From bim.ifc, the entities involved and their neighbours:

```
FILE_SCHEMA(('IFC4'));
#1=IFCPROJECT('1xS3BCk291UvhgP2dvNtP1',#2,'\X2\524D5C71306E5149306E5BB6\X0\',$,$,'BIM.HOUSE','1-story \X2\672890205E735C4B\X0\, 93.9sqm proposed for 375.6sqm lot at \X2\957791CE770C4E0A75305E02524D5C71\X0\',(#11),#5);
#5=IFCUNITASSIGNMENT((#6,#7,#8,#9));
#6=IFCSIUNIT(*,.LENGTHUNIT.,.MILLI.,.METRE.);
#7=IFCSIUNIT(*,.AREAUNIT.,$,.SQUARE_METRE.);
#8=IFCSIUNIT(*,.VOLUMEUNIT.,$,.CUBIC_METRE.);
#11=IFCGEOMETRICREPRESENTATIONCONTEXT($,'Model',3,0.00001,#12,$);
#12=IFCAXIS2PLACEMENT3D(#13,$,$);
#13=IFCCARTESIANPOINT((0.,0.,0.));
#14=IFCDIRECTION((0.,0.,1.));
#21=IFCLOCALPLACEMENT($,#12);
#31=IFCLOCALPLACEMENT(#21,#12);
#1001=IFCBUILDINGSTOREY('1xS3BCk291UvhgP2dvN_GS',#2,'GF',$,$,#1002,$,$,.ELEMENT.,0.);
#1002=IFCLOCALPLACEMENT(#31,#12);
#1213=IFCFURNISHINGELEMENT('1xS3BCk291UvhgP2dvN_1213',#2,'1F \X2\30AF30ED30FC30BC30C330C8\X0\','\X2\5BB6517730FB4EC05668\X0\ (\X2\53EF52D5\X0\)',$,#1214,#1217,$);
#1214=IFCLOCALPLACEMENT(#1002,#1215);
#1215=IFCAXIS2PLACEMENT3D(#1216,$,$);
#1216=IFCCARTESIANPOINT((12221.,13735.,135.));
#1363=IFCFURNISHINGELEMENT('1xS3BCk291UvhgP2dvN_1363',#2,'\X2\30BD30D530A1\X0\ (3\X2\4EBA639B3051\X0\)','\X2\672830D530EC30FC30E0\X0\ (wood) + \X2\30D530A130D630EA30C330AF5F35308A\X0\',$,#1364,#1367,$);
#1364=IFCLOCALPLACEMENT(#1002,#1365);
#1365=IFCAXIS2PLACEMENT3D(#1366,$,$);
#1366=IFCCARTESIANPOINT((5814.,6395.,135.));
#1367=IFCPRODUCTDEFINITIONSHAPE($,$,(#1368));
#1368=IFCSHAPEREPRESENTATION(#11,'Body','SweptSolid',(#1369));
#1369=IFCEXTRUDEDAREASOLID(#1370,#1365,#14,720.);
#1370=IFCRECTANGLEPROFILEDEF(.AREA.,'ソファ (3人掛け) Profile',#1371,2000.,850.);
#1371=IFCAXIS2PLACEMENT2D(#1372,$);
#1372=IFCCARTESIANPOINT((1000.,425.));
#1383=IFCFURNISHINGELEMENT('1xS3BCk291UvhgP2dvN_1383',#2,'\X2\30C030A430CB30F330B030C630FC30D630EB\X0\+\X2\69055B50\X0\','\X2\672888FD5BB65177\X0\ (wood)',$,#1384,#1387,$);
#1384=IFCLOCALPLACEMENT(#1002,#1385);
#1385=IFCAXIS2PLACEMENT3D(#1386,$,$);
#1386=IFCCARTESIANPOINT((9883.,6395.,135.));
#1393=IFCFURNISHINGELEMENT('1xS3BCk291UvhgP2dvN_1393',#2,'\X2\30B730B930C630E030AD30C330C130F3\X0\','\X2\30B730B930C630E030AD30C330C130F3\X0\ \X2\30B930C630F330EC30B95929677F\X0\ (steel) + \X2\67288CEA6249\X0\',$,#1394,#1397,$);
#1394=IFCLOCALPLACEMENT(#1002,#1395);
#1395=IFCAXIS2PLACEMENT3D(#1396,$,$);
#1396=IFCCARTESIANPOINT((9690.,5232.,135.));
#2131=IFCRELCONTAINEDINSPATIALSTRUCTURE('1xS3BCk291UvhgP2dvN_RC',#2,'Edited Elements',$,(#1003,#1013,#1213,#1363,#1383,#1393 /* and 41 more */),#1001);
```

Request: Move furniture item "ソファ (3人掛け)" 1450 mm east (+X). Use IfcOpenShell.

```python
import ifcopenshell
import ifcopenshell.api.geometry
import ifcopenshell.util.placement
import ifcopenshell.util.unit

model = ifcopenshell.open("bim.ifc")
unit_scale = ifcopenshell.util.unit.calculate_unit_scale(model)

item = model.by_id(1363)
matrix = ifcopenshell.util.placement.get_local_placement(item.ObjectPlacement)
matrix[0, 3] += 1.45 / unit_scale
ifcopenshell.api.geometry.edit_object_placement(model, product=item, matrix=matrix, is_si=False)

print(ifcopenshell.util.placement.get_local_placement(item.ObjectPlacement).round(3) + 0.0)

model.write("bim_edited.ifc")
```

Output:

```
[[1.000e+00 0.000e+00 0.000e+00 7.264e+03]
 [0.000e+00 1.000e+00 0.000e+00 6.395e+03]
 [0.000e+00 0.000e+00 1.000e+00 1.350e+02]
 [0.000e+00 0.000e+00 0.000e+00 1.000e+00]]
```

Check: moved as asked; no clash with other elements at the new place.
